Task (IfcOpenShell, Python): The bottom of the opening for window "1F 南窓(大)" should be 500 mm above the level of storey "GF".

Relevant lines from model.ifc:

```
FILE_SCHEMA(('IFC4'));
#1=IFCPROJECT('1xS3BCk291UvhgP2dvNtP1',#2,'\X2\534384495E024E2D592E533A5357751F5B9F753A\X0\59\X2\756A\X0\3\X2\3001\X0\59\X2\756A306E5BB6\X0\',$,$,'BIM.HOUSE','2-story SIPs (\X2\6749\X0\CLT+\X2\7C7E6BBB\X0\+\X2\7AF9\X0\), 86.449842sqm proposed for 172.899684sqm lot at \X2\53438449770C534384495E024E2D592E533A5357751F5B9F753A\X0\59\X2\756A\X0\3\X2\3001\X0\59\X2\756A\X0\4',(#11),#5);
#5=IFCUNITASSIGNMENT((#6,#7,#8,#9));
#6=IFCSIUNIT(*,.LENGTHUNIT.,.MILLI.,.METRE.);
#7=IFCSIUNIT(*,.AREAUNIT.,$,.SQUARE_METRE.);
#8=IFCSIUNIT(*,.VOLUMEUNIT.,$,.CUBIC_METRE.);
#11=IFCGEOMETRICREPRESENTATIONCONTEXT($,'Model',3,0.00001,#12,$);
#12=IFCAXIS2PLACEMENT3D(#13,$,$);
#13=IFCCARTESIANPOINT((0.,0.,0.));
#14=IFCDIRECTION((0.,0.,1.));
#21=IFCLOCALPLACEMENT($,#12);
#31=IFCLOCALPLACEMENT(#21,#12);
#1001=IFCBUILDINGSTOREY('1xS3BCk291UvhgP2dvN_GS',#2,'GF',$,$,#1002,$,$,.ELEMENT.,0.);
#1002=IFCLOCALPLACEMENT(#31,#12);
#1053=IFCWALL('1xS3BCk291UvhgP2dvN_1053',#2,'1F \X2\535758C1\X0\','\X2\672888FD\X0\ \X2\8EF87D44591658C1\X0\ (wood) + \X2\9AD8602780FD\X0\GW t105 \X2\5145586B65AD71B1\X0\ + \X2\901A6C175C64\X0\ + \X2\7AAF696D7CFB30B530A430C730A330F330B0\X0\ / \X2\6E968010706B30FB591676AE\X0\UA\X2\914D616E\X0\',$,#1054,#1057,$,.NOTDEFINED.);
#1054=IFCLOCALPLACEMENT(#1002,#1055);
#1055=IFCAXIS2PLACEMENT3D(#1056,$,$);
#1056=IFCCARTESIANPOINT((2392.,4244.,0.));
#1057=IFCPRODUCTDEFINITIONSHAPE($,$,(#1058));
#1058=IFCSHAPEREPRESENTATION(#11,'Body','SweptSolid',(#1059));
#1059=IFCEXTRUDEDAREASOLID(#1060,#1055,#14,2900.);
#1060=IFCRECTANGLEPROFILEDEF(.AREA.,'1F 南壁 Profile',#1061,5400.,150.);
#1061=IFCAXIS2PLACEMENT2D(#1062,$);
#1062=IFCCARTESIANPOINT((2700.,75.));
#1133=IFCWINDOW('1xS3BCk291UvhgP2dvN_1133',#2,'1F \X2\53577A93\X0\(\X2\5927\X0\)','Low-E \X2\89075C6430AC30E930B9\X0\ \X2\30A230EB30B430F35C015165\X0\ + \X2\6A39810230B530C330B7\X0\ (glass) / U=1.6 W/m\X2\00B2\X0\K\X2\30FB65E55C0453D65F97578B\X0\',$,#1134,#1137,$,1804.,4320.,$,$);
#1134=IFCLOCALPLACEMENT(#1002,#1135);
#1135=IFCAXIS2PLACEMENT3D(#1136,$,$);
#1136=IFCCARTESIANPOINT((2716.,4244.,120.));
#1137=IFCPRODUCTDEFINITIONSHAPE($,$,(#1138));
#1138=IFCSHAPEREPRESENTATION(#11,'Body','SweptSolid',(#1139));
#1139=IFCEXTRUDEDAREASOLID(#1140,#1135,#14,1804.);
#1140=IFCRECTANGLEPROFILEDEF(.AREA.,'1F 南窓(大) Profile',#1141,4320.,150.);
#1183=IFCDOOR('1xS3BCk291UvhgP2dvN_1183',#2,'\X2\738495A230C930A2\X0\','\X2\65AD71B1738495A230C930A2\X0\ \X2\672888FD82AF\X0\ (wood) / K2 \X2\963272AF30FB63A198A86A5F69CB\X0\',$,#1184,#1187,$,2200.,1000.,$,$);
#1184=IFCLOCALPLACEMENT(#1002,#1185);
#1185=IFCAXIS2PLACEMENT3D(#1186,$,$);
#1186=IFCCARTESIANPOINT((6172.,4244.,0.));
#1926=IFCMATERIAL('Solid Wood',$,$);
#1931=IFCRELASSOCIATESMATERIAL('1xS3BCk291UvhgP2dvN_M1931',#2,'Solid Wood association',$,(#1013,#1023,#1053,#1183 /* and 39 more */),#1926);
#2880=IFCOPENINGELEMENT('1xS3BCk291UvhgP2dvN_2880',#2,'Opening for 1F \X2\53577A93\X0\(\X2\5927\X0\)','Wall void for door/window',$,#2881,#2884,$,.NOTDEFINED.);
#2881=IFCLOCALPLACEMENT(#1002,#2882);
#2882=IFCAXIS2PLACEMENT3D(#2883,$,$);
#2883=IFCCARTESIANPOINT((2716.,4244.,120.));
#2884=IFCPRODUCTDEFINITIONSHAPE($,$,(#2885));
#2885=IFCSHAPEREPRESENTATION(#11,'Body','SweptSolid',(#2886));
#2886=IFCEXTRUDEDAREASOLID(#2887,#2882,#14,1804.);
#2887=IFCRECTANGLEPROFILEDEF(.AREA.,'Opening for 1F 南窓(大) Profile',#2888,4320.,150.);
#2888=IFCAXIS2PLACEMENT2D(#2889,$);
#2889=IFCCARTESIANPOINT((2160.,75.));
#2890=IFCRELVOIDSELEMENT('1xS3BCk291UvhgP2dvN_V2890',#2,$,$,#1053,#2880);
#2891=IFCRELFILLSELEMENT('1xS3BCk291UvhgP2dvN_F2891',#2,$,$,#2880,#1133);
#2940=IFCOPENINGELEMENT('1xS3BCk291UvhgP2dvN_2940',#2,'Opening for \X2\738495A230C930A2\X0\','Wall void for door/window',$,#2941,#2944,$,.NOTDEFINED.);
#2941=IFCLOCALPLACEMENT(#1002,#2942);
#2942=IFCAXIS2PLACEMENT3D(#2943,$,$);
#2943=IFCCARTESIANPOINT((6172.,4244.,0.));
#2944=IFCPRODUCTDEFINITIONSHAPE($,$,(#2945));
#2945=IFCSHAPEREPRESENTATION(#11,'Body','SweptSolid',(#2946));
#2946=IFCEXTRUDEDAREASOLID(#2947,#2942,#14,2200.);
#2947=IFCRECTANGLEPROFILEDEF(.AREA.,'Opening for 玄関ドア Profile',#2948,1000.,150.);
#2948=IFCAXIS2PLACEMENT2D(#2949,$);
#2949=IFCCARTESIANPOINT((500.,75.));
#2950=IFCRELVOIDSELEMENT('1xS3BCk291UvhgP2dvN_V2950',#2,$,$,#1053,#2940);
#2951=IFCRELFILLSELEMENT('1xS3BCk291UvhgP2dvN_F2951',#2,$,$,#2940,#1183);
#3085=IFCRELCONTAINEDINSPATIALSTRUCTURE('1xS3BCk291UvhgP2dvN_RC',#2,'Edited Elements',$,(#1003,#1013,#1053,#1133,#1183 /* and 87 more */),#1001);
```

```python
import numpy as np
import ifcopenshell
import ifcopenshell.api.geometry
import ifcopenshell.geom
import ifcopenshell.util.element
import ifcopenshell.util.placement
import ifcopenshell.util.shape
import ifcopenshell.util.unit

model = ifcopenshell.open("model.ifc")
unit_scale = ifcopenshell.util.unit.calculate_unit_scale(model)

window = model.by_id(1133)
opening = window.FillsVoids[0].RelatingOpeningElement
storey = ifcopenshell.util.element.get_container(window, ifc_class="IfcBuildingStorey")
level = ifcopenshell.util.placement.get_local_placement(storey.ObjectPlacement)[2, 3]

# The opening's origin need not be at the sill, so measure its lowest point.
shape = ifcopenshell.geom.create_shape(ifcopenshell.geom.settings(), opening)
bottom = ifcopenshell.util.shape.get_shape_bottom_elevation(shape, shape.geometry) / unit_scale
dz = level + 500.0 - bottom

shift = np.array([0.0, 0.0, dz])
# The window is not placed relative to its opening, so move both.
for product in (opening, window):
    matrix = ifcopenshell.util.placement.get_local_placement(product.ObjectPlacement)
    matrix[:3, 3] += shift
    ifcopenshell.api.geometry.edit_object_placement(model, product=product, matrix=matrix, is_si=False)

print(f"moved by {dz * unit_scale:+.3f} m")

model.write("model_rev.ifc")
```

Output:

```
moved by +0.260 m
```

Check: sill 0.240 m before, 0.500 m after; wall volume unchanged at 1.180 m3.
